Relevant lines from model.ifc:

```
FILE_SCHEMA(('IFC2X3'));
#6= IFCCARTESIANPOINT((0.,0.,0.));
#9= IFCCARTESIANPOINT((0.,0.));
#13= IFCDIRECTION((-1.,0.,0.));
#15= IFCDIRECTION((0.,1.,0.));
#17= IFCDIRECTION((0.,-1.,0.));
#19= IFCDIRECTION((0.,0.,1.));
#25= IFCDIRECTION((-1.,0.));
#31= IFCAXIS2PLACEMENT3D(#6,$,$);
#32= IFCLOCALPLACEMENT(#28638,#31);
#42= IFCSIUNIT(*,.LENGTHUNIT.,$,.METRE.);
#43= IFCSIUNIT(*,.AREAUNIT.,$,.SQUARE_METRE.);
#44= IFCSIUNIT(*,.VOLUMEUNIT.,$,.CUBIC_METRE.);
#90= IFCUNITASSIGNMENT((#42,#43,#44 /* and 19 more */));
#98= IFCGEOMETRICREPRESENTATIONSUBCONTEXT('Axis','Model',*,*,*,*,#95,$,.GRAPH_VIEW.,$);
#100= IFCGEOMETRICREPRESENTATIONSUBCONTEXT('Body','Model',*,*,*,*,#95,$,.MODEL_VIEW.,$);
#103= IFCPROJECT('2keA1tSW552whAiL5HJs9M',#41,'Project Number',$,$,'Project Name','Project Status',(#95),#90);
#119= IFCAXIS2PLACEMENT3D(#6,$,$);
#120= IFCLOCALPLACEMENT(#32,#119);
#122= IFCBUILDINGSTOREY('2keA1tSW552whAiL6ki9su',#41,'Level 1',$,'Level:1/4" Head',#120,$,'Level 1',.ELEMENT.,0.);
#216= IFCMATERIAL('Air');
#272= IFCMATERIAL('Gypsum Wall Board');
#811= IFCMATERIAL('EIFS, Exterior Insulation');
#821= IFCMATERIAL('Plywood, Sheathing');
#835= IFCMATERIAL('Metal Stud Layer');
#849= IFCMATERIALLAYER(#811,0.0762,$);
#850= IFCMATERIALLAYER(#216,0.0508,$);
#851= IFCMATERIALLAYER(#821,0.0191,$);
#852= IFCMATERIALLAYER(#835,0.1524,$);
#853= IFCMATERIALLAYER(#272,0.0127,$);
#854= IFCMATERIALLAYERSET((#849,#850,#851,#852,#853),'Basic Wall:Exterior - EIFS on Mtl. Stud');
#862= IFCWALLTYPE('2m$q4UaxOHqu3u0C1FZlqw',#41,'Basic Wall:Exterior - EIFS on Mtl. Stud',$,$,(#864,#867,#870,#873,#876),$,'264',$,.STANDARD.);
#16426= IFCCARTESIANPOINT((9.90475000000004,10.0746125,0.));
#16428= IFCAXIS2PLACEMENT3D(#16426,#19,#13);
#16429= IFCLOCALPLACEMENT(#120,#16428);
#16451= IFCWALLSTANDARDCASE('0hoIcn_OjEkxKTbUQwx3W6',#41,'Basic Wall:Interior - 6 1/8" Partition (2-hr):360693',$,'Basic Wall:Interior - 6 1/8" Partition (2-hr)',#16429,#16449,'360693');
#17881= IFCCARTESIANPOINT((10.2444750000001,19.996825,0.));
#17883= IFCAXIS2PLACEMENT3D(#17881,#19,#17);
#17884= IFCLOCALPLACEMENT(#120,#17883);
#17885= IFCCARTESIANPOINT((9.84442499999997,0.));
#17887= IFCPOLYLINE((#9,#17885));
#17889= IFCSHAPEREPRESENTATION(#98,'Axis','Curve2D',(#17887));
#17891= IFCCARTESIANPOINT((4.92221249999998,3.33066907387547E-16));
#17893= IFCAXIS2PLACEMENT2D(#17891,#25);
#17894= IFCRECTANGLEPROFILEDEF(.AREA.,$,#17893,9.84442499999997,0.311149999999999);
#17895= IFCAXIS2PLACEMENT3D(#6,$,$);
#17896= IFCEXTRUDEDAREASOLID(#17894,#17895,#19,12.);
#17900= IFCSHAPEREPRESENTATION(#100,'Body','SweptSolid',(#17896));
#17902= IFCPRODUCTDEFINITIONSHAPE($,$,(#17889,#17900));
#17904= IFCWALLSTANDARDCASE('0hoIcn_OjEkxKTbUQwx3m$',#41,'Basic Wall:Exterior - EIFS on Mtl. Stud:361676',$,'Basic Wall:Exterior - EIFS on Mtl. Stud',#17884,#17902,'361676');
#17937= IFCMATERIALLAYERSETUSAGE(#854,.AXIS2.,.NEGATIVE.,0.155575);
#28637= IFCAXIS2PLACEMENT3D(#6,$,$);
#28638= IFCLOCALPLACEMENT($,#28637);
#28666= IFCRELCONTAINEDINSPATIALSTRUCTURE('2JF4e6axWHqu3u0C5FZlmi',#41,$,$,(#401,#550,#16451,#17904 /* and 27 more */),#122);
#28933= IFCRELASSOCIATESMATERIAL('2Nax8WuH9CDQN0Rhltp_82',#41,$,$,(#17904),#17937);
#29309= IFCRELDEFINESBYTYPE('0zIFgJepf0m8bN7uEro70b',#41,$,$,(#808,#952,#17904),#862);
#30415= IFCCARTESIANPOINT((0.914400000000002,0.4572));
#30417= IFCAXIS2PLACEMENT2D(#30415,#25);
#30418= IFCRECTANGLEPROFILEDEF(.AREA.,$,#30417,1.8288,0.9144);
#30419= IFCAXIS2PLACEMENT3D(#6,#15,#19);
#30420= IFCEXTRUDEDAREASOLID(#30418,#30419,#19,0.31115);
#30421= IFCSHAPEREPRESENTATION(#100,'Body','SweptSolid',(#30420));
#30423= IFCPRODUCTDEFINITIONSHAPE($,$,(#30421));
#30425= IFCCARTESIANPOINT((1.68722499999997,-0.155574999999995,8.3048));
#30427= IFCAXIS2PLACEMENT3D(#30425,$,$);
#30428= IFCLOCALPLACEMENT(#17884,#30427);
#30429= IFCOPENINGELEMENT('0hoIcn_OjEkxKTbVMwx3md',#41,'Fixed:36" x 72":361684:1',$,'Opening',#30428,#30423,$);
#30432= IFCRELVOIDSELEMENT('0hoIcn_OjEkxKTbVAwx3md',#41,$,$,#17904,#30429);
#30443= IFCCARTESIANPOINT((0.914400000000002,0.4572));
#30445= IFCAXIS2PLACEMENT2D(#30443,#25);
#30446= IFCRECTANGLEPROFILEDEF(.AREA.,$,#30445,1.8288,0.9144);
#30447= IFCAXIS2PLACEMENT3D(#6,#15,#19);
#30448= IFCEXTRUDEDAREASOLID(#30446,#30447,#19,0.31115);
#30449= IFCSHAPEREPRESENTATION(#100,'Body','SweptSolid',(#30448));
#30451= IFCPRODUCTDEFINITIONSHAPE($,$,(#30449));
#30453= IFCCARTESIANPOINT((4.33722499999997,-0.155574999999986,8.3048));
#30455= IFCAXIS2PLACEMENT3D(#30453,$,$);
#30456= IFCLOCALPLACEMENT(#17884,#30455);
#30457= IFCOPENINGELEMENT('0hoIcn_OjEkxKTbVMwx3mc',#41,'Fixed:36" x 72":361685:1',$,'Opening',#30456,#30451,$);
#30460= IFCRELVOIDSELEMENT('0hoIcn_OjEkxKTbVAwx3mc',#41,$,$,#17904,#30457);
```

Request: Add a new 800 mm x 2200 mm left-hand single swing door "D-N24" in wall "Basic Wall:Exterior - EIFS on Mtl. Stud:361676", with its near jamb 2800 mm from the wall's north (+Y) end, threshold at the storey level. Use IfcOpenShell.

```python
import numpy as np
import ifcopenshell
import ifcopenshell.api.feature
import ifcopenshell.api.geometry
import ifcopenshell.api.root
import ifcopenshell.api.spatial
import ifcopenshell.api.type
import ifcopenshell.geom
import ifcopenshell.util.element
import ifcopenshell.util.placement
import ifcopenshell.util.representation
import ifcopenshell.util.shape
import ifcopenshell.util.unit

model = ifcopenshell.open("model.ifc")
unit_scale = ifcopenshell.util.unit.calculate_unit_scale(model)
settings = ifcopenshell.geom.settings()


def volume(element):
    """Net volume in cubic metres, openings subtracted."""
    shape = ifcopenshell.geom.create_shape(settings, element)
    return ifcopenshell.util.shape.get_volume(shape.geometry)


wall = model.by_guid("0hoIcn_OjEkxKTbUQwx3m$")
storey = ifcopenshell.util.element.get_container(wall, ifc_class="IfcBuildingStorey")
context = ifcopenshell.util.representation.get_context(model, "Model", "Body", "MODEL_VIEW")
before = volume(wall)

width, height, from_end, sill = 0.8, 2.2, 2.8, 0.0  # metres

# The wall runs along its own X axis, and the end named is its -X end.
wall_shape = ifcopenshell.geom.create_shape(settings, wall)
x, y, z = ifcopenshell.util.shape.get_vertices(wall_shape.geometry).T
start = x.min() + from_end
face, thickness = float(y.min()), float(y.max() - y.min())
wall_matrix = ifcopenshell.util.placement.get_local_placement(wall.ObjectPlacement)
level = ifcopenshell.util.placement.get_local_placement(storey.ObjectPlacement)[2, 3]


def in_wall(x, y):
    """Placement at x, y metres in the wall's axes, at sill height."""
    matrix = wall_matrix.copy()
    matrix[:, 3] = wall_matrix @ np.array([x / unit_scale, y / unit_scale, 0.0, 1.0])
    matrix[2, 3] = level + sill / unit_scale
    return matrix


# Opening: a box that overshoots both wall faces by 50 mm.
opening = ifcopenshell.api.root.create_entity(model, ifc_class="IfcOpeningElement")
box = ifcopenshell.api.geometry.add_wall_representation(
    model, context=context, length=width, height=height, thickness=thickness + 0.1
)
ifcopenshell.api.geometry.assign_representation(model, product=opening, representation=box)
ifcopenshell.api.geometry.edit_object_placement(model, product=opening, matrix=in_wall(start, face - 0.05), is_si=False)
ifcopenshell.api.feature.add_feature(model, feature=opening, element=wall)

door = ifcopenshell.api.root.create_entity(model, ifc_class="IfcDoor", name="D-N24")
door.OverallWidth, door.OverallHeight = width / unit_scale, height / unit_scale
body = ifcopenshell.api.geometry.add_door_representation(
    model,
    context=context,
    overall_width=door.OverallWidth,
    overall_height=door.OverallHeight,
    operation_type="SINGLE_SWING_LEFT",
    lining_properties={"LiningDepth": thickness / unit_scale, "ThresholdDepth": thickness / unit_scale},
)
ifcopenshell.api.geometry.assign_representation(model, product=door, representation=body)
ifcopenshell.api.spatial.assign_container(model, products=[door], relating_structure=storey)
fills = ifcopenshell.api.feature.add_filling(model, opening=opening, element=door)
fills.OwnerHistory = door.OwnerHistory  # required in IFC2X3

# IFC2X3 keeps the operation on the door style.
style = ifcopenshell.api.root.create_entity(model, ifc_class="IfcDoorStyle", name="D-N24")
style.OperationType, style.ConstructionType = "SINGLE_SWING_LEFT", "NOTDEFINED"
style.ParameterTakesPrecedence = style.Sizeable = False
ifcopenshell.api.type.assign_type(model, related_objects=[door], relating_type=style)

# The lining spans the wall, so the door starts at the wall face.
ifcopenshell.api.geometry.edit_object_placement(model, product=door, matrix=in_wall(start, face), is_si=False)

after = volume(wall)

print(f"wall volume {before:.3f} -> {after:.3f} m3")

model.write("model_updated.ifc")
```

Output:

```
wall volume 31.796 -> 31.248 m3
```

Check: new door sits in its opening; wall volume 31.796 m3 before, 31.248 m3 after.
